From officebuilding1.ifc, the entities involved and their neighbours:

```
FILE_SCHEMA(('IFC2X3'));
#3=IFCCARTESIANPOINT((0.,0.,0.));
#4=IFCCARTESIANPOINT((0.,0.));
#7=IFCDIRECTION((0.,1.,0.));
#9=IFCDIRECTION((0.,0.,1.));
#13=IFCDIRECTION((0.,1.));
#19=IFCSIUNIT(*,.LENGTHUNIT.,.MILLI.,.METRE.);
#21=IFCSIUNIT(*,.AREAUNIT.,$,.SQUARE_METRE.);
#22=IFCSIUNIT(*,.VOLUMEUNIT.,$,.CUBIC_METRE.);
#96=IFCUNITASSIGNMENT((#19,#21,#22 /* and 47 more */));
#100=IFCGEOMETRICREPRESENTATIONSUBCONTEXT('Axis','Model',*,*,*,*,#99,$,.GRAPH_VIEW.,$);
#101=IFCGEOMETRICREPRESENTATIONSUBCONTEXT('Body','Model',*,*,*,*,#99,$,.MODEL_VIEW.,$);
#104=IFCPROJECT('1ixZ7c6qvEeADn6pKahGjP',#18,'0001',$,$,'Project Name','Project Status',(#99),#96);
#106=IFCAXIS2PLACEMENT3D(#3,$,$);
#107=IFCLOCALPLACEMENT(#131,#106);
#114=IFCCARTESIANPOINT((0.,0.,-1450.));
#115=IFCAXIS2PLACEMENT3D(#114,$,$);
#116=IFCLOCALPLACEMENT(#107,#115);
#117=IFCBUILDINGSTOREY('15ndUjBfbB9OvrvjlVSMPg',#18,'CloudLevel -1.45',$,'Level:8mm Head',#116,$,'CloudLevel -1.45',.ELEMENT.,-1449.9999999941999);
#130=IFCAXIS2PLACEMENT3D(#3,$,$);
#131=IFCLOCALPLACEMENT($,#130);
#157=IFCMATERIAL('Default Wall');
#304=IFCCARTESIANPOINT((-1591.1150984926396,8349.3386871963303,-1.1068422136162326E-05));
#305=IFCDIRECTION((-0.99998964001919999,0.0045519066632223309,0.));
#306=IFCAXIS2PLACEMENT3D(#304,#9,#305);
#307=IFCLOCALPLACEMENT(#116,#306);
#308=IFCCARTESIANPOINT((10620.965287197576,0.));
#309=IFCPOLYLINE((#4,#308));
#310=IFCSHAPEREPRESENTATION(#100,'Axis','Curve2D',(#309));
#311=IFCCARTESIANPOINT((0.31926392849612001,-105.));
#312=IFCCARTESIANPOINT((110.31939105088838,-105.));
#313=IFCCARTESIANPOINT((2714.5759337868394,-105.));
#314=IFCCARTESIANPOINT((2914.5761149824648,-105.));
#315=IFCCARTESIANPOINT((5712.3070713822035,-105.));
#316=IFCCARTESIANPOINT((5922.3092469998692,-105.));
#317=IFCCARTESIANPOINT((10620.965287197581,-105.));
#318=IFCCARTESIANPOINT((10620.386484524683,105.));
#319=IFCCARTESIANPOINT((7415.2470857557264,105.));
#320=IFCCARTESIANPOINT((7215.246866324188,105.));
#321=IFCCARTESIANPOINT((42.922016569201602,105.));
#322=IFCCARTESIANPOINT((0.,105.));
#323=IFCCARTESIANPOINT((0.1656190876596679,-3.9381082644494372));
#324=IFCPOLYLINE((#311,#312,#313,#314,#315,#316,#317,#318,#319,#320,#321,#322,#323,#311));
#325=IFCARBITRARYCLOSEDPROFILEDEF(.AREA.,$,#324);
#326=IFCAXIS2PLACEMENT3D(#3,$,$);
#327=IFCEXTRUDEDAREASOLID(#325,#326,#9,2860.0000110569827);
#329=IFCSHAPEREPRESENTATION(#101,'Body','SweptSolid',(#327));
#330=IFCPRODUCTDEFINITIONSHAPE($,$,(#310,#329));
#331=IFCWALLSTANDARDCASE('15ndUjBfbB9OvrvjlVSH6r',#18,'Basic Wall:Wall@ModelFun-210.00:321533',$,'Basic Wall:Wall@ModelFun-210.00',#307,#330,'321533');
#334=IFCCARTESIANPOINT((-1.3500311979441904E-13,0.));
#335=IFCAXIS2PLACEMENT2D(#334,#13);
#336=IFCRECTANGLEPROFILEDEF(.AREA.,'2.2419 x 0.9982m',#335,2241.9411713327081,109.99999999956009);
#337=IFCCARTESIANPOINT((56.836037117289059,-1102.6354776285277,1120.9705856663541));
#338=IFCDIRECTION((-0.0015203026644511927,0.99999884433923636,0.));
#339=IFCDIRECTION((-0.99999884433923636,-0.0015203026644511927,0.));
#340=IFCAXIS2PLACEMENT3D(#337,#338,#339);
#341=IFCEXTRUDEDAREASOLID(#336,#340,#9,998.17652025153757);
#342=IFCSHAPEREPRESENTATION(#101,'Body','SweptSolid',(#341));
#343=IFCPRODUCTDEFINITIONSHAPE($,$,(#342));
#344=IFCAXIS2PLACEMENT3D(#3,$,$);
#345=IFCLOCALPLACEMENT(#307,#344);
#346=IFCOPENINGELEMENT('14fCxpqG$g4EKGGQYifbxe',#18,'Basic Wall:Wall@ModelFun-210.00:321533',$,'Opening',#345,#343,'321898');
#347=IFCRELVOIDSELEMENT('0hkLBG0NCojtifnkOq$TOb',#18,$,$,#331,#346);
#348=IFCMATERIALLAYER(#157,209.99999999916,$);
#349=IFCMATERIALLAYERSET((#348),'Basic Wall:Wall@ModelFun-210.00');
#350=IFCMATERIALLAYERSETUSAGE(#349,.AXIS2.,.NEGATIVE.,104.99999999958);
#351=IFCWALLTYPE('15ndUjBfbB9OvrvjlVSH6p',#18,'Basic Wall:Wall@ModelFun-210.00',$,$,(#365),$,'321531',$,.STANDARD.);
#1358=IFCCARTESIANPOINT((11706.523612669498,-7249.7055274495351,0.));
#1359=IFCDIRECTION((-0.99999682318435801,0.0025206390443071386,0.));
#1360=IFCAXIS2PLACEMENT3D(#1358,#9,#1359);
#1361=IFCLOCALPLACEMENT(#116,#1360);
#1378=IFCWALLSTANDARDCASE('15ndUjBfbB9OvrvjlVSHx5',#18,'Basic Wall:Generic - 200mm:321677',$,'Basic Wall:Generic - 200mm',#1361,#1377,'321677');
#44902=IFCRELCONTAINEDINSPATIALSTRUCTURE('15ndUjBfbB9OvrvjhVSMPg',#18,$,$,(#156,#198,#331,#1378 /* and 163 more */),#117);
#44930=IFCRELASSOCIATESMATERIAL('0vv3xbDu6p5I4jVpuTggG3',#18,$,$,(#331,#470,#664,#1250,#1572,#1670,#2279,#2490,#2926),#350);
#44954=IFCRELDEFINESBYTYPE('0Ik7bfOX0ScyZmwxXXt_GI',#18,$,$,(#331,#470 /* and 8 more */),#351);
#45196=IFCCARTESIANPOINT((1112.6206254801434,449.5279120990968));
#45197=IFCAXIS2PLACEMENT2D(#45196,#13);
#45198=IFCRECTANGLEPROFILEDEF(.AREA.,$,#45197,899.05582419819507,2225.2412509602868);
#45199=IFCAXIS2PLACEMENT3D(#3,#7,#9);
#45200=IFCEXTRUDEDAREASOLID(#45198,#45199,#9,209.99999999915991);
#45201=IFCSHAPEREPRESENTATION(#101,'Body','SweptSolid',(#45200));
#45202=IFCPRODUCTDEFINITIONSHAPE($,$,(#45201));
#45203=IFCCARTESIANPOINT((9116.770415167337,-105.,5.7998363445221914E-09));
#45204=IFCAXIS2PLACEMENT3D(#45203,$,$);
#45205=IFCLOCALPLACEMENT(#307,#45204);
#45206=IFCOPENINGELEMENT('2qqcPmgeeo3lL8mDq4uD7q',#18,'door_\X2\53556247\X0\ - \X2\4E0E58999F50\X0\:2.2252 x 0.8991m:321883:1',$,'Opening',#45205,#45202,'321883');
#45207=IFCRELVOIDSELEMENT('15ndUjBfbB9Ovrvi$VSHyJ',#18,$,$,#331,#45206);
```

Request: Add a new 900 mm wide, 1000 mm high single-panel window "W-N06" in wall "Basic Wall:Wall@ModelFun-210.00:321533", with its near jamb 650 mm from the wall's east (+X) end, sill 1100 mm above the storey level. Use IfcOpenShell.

```python
import numpy as np
import ifcopenshell
import ifcopenshell.api.feature
import ifcopenshell.api.geometry
import ifcopenshell.api.root
import ifcopenshell.api.spatial
import ifcopenshell.api.type
import ifcopenshell.geom
import ifcopenshell.util.element
import ifcopenshell.util.placement
import ifcopenshell.util.representation
import ifcopenshell.util.shape
import ifcopenshell.util.unit

model = ifcopenshell.open("officebuilding1.ifc")
unit_scale = ifcopenshell.util.unit.calculate_unit_scale(model)
settings = ifcopenshell.geom.settings()


def volume(element):
    """Net volume in cubic metres, openings subtracted."""
    shape = ifcopenshell.geom.create_shape(settings, element)
    return ifcopenshell.util.shape.get_volume(shape.geometry)


wall = model.by_guid("15ndUjBfbB9OvrvjlVSH6r")
storey = ifcopenshell.util.element.get_container(wall, ifc_class="IfcBuildingStorey")
context = ifcopenshell.util.representation.get_context(model, "Model", "Body", "MODEL_VIEW")
before = volume(wall)

width, height, from_end, sill = 0.9, 1, 0.65, 1.1  # metres

# The wall runs along its own X axis, and the end named is its -X end.
wall_shape = ifcopenshell.geom.create_shape(settings, wall)
x, y, z = ifcopenshell.util.shape.get_vertices(wall_shape.geometry).T
start = x.min() + from_end
face, thickness = float(y.min()), float(y.max() - y.min())
wall_matrix = ifcopenshell.util.placement.get_local_placement(wall.ObjectPlacement)
level = ifcopenshell.util.placement.get_local_placement(storey.ObjectPlacement)[2, 3]


def in_wall(x, y):
    """Placement at x, y metres in the wall's axes, at sill height."""
    matrix = wall_matrix.copy()
    matrix[:, 3] = wall_matrix @ np.array([x / unit_scale, y / unit_scale, 0.0, 1.0])
    matrix[2, 3] = level + sill / unit_scale
    return matrix


# Opening: a box that overshoots both wall faces by 50 mm.
opening = ifcopenshell.api.root.create_entity(model, ifc_class="IfcOpeningElement")
box = ifcopenshell.api.geometry.add_wall_representation(
    model, context=context, length=width, height=height, thickness=thickness + 0.1
)
ifcopenshell.api.geometry.assign_representation(model, product=opening, representation=box)
ifcopenshell.api.geometry.edit_object_placement(model, product=opening, matrix=in_wall(start, face - 0.05), is_si=False)
ifcopenshell.api.feature.add_feature(model, feature=opening, element=wall)

window = ifcopenshell.api.root.create_entity(model, ifc_class="IfcWindow", name="W-N06")
window.OverallWidth, window.OverallHeight = width / unit_scale, height / unit_scale
body = ifcopenshell.api.geometry.add_window_representation(
    model,
    context=context,
    overall_width=window.OverallWidth,
    overall_height=window.OverallHeight,
    partition_type="SINGLE_PANEL",
)
ifcopenshell.api.geometry.assign_representation(model, product=window, representation=body)
ifcopenshell.api.spatial.assign_container(model, products=[window], relating_structure=storey)
fills = ifcopenshell.api.feature.add_filling(model, opening=opening, element=window)
fills.OwnerHistory = window.OwnerHistory  # required in IFC2X3

# IFC2X3 keeps the operation on the window style.
style = ifcopenshell.api.root.create_entity(model, ifc_class="IfcWindowStyle", name="W-N06")
style.OperationType, style.ConstructionType = "SINGLE_PANEL", "NOTDEFINED"
style.ParameterTakesPrecedence = style.Sizeable = False
ifcopenshell.api.type.assign_type(model, related_objects=[window], relating_type=style)

# Centre the window in the wall's thickness.
ifcopenshell.api.geometry.edit_object_placement(model, product=window, matrix=in_wall(start, face), is_si=False)
window_shape = ifcopenshell.geom.create_shape(settings, window)
depth = ifcopenshell.util.shape.get_vertices(window_shape.geometry)[:, 1]
offset = face + thickness / 2 - (depth.min() + depth.max()) / 2
ifcopenshell.api.geometry.edit_object_placement(model, product=window, matrix=in_wall(start, offset), is_si=False)

after = volume(wall)

print(f"wall volume {before:.3f} -> {after:.3f} m3")

model.write("officebuilding1_updated.ifc")
```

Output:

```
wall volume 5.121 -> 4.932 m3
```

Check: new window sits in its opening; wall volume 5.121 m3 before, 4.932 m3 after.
